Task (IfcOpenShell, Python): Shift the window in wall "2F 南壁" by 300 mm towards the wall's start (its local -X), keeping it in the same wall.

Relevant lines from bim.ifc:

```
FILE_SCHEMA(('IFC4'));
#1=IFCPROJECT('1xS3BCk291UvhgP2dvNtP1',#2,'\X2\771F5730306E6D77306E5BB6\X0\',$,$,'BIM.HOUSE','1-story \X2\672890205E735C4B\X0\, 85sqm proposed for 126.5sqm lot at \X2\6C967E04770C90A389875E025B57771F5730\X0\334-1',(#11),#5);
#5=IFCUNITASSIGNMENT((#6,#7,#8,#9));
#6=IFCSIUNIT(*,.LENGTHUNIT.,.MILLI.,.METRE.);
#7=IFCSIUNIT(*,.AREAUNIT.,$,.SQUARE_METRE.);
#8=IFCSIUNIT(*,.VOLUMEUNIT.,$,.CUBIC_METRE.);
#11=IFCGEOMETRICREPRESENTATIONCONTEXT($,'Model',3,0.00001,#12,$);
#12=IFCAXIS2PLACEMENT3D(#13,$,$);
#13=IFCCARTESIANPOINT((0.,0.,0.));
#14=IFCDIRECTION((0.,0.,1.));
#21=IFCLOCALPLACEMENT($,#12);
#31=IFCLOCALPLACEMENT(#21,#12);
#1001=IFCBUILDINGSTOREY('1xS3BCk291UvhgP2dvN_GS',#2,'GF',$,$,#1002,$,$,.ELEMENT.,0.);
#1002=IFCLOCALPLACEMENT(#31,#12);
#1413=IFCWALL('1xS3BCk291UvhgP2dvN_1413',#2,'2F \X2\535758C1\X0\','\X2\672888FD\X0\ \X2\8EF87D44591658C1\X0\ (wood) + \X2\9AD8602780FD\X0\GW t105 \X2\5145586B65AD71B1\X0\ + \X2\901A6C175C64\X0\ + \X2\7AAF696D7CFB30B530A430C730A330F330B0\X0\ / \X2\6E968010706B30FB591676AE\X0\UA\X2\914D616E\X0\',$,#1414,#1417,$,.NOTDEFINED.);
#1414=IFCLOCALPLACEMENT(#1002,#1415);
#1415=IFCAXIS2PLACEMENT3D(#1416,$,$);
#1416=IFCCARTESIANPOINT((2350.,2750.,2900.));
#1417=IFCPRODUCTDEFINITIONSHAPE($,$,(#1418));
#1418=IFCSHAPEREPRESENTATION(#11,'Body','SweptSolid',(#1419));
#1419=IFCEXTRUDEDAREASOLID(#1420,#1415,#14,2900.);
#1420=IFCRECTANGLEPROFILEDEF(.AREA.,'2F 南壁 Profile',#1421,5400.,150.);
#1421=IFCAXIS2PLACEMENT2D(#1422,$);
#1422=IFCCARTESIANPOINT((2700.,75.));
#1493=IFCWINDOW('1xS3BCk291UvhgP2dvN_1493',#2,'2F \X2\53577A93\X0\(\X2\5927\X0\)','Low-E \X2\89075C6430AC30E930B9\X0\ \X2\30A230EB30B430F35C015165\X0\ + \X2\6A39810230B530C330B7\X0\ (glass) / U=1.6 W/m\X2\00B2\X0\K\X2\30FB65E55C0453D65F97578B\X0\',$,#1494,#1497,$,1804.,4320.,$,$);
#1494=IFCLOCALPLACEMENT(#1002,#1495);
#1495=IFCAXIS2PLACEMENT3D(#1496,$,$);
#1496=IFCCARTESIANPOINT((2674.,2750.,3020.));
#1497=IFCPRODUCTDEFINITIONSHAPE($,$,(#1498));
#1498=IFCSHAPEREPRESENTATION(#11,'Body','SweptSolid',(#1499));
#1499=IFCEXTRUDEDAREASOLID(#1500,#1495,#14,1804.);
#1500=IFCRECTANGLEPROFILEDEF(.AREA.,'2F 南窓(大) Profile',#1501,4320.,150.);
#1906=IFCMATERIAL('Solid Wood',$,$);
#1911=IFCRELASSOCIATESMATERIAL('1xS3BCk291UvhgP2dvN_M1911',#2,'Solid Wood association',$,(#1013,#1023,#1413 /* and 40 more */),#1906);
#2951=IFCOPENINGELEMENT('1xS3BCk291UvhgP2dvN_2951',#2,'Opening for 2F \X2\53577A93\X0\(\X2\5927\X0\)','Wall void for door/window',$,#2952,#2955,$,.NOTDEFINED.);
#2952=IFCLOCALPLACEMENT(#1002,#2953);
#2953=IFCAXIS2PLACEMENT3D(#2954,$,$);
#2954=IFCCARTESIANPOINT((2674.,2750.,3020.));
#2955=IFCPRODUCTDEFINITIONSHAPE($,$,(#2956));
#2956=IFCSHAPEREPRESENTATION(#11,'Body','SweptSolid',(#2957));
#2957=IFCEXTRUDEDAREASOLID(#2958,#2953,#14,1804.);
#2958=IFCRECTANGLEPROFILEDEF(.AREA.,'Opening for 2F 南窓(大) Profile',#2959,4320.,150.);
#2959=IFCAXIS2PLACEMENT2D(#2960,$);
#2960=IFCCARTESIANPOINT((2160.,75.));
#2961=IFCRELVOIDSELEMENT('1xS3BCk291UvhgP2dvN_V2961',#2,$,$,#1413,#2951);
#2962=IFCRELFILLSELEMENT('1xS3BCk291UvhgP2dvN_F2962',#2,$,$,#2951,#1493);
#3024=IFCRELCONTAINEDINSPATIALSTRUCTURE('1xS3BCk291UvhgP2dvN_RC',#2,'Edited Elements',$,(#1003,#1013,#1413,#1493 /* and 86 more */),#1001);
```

```python
import ifcopenshell
import ifcopenshell.api.geometry
import ifcopenshell.util.placement
import ifcopenshell.util.unit

model = ifcopenshell.open("bim.ifc")
unit_scale = ifcopenshell.util.unit.calculate_unit_scale(model)

window = model.by_guid("1xS3BCk291UvhgP2dvN_1493")
opening = window.FillsVoids[0].RelatingOpeningElement
wall = opening.VoidsElements[0].RelatingBuildingElement

wall_matrix = ifcopenshell.util.placement.get_local_placement(wall.ObjectPlacement)
shift = wall_matrix[:3, 0] * -0.3 / unit_scale
before = ifcopenshell.util.placement.get_local_placement(window.ObjectPlacement)[:3, 3].copy()

# The window is not placed relative to its opening, so move both.
for product in (opening, window):
    matrix = ifcopenshell.util.placement.get_local_placement(product.ObjectPlacement)
    matrix[:3, 3] += shift
    ifcopenshell.api.geometry.edit_object_placement(model, product=product, matrix=matrix, is_si=False)

after = ifcopenshell.util.placement.get_local_placement(window.ObjectPlacement)[:3, 3]
print("window moved by", (after - before).round(3) + 0.0)

model.write("bim_v2.ifc")
```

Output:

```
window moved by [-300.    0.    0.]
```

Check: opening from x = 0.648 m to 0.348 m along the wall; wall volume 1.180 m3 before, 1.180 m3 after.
